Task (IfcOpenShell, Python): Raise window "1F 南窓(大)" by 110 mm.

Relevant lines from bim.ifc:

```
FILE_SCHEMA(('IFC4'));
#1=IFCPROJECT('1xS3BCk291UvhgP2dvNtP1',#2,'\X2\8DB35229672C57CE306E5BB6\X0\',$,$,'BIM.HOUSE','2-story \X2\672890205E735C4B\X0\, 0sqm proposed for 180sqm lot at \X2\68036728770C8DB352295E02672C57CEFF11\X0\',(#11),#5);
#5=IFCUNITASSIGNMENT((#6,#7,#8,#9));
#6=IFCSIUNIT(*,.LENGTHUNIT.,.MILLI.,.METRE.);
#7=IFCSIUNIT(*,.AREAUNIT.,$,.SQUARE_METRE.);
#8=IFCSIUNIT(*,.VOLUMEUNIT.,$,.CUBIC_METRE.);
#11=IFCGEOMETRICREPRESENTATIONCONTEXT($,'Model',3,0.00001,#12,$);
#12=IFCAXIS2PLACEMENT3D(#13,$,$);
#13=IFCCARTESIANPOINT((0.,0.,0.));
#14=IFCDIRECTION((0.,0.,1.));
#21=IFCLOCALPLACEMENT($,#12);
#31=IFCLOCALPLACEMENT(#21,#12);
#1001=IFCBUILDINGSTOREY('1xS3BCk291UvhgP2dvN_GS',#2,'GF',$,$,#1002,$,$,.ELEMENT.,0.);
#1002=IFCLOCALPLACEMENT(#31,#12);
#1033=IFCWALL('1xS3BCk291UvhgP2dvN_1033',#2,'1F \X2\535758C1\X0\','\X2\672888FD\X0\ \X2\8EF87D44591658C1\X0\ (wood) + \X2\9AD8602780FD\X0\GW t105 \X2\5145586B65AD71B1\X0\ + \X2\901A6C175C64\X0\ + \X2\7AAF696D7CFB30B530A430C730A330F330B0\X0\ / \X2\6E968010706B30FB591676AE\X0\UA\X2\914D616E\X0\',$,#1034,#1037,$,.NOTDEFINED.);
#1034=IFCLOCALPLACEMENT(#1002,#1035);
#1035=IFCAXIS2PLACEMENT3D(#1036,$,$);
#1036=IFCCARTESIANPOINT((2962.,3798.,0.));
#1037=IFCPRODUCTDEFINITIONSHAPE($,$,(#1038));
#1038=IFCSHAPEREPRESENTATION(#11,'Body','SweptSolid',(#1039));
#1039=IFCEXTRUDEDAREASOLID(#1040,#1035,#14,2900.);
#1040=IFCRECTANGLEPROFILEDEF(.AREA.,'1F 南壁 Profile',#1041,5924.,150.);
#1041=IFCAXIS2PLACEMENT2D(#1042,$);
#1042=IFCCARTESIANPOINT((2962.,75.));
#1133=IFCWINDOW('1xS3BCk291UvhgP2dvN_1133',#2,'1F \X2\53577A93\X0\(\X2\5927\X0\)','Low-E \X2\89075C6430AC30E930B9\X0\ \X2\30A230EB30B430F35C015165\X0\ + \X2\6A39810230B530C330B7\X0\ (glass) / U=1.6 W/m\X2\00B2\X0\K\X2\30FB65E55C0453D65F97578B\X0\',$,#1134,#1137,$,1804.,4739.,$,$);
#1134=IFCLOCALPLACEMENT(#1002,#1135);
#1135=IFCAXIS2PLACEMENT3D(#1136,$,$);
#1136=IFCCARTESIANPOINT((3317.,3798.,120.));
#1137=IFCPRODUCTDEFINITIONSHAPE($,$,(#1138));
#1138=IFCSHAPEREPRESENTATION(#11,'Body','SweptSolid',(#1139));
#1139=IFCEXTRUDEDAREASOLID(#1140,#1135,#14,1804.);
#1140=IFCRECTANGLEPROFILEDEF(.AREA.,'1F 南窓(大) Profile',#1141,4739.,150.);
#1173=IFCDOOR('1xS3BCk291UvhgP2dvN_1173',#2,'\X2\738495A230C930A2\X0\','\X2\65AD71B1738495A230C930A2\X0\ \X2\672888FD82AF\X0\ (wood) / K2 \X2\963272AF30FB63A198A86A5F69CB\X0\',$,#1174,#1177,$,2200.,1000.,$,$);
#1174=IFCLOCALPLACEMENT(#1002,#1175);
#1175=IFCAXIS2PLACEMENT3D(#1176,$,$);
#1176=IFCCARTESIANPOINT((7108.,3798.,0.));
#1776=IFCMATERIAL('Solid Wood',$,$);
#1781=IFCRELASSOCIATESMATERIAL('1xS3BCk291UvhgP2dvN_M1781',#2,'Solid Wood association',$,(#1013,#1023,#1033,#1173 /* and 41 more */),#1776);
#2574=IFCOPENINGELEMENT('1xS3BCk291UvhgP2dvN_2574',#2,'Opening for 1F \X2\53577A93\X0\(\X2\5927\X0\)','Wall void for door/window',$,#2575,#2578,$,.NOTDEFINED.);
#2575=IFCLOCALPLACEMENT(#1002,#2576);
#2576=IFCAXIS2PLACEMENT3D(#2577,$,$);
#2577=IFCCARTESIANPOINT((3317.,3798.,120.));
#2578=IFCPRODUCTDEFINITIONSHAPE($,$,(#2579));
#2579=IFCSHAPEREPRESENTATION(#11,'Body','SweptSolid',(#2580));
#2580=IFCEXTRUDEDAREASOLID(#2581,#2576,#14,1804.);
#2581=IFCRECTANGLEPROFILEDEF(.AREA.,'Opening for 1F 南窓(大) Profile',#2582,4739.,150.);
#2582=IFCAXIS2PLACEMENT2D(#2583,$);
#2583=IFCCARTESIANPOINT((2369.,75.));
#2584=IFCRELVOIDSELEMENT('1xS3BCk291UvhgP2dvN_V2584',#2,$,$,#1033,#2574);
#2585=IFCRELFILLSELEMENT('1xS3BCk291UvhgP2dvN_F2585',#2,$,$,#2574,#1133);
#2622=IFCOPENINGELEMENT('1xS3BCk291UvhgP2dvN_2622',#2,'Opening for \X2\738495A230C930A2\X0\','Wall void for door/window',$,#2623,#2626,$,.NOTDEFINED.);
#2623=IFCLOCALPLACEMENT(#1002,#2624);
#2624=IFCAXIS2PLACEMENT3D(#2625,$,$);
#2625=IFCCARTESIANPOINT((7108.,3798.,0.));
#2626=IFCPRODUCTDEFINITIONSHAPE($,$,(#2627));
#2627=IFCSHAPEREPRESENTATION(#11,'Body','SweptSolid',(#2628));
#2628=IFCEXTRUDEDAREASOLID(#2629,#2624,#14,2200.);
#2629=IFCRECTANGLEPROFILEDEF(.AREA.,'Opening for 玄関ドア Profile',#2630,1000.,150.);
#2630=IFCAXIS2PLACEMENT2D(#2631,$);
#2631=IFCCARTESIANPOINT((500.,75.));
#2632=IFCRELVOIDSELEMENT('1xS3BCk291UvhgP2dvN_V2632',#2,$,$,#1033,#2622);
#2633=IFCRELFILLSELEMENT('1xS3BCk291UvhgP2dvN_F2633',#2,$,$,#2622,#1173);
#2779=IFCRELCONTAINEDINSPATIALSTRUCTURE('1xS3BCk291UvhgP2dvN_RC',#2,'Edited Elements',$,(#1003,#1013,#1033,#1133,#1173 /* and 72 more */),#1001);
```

```python
import numpy as np
import ifcopenshell
import ifcopenshell.api.geometry
import ifcopenshell.util.placement
import ifcopenshell.util.unit

model = ifcopenshell.open("bim.ifc")
unit_scale = ifcopenshell.util.unit.calculate_unit_scale(model)

window = model.by_guid("1xS3BCk291UvhgP2dvN_1133")
opening = window.FillsVoids[0].RelatingOpeningElement
dz = 0.11 / unit_scale

shift = np.array([0.0, 0.0, dz])
# The window is not placed relative to its opening, so move both.
for product in (opening, window):
    matrix = ifcopenshell.util.placement.get_local_placement(product.ObjectPlacement)
    matrix[:3, 3] += shift
    ifcopenshell.api.geometry.edit_object_placement(model, product=product, matrix=matrix, is_si=False)

print(f"moved by {dz * unit_scale:+.3f} m")

model.write("bim_rev.ifc")
```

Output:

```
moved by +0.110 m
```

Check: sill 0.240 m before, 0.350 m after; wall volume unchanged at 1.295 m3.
